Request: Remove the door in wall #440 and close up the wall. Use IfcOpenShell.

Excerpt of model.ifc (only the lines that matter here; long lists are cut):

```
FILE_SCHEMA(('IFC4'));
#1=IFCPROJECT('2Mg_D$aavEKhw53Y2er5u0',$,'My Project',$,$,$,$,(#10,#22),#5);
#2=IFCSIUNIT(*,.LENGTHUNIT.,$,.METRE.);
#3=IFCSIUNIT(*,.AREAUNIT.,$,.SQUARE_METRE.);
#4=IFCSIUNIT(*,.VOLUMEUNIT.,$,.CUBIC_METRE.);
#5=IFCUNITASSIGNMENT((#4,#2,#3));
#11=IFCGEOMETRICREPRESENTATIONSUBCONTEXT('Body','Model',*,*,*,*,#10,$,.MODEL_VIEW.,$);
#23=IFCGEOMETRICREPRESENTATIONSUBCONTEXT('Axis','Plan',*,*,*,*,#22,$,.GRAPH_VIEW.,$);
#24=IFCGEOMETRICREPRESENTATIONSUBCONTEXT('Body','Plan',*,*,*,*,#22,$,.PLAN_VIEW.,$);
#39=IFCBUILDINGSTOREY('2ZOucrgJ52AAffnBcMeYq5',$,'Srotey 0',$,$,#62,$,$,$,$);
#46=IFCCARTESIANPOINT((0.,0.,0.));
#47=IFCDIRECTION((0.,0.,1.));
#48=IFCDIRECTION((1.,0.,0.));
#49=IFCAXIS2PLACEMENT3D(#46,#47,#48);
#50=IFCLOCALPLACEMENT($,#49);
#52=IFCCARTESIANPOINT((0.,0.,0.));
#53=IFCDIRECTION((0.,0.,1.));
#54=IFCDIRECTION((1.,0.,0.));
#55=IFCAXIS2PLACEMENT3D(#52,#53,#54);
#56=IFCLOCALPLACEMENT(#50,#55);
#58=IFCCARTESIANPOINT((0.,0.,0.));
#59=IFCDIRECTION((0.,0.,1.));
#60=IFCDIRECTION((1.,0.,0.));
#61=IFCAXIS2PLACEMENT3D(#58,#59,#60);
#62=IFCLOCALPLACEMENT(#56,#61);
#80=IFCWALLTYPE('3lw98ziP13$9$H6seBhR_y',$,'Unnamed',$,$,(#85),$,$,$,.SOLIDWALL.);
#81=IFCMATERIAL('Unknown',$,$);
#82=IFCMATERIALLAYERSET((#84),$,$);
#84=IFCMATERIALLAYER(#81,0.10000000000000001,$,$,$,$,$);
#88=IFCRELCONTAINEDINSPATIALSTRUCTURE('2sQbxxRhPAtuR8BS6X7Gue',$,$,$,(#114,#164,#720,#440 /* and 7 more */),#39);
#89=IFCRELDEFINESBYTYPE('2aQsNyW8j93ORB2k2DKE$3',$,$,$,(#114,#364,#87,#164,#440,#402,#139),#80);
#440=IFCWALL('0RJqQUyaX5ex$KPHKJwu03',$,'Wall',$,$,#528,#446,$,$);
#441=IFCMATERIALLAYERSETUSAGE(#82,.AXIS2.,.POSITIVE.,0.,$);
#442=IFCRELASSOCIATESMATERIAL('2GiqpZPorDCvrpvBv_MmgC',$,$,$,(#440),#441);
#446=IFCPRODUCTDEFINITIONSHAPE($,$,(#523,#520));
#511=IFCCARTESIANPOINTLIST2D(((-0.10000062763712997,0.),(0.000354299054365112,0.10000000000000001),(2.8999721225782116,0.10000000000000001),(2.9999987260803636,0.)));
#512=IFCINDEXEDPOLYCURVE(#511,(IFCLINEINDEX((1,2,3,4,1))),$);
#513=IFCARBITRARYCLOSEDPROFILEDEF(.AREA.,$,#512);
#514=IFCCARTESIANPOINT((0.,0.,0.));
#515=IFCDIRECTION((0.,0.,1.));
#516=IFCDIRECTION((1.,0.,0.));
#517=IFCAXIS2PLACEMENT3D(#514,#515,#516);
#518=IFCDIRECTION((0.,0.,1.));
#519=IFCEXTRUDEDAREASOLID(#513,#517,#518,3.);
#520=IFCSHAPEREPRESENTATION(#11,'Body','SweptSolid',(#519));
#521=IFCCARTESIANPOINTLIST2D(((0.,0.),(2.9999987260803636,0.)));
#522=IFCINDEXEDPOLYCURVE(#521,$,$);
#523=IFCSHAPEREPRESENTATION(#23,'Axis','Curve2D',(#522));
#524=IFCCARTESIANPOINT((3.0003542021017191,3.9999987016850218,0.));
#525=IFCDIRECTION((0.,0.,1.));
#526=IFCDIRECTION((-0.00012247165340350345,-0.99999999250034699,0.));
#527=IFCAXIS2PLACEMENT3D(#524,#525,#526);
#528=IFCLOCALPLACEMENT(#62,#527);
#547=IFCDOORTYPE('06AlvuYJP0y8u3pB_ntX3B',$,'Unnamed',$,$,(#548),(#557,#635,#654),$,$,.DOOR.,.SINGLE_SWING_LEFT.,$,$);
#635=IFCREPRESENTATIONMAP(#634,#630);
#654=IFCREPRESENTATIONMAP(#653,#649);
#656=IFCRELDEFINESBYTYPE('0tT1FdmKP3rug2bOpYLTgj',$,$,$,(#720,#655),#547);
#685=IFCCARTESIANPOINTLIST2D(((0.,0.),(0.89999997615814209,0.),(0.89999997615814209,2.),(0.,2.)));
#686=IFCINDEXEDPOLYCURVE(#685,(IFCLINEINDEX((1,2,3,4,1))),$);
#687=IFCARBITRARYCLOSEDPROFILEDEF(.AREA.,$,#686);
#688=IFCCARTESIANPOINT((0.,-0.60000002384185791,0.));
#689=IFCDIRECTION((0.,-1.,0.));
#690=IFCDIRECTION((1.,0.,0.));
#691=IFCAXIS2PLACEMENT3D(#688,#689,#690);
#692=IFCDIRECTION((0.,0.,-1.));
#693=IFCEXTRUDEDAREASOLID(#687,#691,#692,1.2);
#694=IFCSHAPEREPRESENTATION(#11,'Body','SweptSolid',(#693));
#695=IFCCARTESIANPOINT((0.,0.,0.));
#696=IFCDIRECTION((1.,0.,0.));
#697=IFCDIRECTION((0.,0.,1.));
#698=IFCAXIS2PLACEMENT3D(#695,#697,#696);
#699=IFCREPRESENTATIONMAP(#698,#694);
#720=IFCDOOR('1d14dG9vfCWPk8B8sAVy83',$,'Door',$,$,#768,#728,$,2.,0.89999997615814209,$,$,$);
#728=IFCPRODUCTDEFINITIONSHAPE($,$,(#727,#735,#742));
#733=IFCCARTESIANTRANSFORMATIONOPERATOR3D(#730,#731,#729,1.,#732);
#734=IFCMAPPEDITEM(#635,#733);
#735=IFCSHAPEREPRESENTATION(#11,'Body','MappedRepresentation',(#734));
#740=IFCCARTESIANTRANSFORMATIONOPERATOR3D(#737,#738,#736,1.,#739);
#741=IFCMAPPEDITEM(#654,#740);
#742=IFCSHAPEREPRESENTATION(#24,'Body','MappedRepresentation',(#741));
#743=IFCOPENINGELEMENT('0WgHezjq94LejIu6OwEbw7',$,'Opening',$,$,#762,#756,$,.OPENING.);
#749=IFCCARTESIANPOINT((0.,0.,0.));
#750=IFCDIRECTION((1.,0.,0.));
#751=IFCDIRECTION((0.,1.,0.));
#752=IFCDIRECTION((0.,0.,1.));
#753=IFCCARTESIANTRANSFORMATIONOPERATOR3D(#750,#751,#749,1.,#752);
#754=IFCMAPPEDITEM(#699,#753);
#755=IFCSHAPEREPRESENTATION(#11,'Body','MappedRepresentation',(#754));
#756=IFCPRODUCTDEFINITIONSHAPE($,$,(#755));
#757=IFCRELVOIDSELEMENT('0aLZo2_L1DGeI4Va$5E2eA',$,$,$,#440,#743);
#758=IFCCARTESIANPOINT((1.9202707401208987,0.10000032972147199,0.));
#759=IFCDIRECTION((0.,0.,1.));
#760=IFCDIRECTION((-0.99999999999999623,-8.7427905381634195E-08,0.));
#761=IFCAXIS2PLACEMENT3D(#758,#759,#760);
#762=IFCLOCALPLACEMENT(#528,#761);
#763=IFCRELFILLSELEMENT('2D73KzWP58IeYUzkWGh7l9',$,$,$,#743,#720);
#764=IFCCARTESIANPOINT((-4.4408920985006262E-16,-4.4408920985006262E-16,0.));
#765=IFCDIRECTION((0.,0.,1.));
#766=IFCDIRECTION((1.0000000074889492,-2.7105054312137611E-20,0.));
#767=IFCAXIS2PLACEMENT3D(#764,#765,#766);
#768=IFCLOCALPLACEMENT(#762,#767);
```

```python
import ifcopenshell
import ifcopenshell.api.feature
import ifcopenshell.api.root
import ifcopenshell.geom
import ifcopenshell.util.shape

model = ifcopenshell.open("model.ifc")
settings = ifcopenshell.geom.settings()


def volume(element):
    """Net volume in cubic metres, openings subtracted."""
    shape = ifcopenshell.geom.create_shape(settings, element)
    return ifcopenshell.util.shape.get_volume(shape.geometry)


door = model.by_id(720)
opening = door.FillsVoids[0].RelatingOpeningElement
wall = opening.VoidsElements[0].RelatingBuildingElement
before = volume(wall)

ifcopenshell.api.root.remove_product(model, product=door)
ifcopenshell.api.feature.remove_feature(model, feature=opening)

after = volume(wall)

print(f"wall volume {before:.3f} -> {after:.3f} m3")

model.write("model-out.ifc")
```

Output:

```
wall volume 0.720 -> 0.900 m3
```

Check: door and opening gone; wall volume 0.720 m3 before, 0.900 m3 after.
